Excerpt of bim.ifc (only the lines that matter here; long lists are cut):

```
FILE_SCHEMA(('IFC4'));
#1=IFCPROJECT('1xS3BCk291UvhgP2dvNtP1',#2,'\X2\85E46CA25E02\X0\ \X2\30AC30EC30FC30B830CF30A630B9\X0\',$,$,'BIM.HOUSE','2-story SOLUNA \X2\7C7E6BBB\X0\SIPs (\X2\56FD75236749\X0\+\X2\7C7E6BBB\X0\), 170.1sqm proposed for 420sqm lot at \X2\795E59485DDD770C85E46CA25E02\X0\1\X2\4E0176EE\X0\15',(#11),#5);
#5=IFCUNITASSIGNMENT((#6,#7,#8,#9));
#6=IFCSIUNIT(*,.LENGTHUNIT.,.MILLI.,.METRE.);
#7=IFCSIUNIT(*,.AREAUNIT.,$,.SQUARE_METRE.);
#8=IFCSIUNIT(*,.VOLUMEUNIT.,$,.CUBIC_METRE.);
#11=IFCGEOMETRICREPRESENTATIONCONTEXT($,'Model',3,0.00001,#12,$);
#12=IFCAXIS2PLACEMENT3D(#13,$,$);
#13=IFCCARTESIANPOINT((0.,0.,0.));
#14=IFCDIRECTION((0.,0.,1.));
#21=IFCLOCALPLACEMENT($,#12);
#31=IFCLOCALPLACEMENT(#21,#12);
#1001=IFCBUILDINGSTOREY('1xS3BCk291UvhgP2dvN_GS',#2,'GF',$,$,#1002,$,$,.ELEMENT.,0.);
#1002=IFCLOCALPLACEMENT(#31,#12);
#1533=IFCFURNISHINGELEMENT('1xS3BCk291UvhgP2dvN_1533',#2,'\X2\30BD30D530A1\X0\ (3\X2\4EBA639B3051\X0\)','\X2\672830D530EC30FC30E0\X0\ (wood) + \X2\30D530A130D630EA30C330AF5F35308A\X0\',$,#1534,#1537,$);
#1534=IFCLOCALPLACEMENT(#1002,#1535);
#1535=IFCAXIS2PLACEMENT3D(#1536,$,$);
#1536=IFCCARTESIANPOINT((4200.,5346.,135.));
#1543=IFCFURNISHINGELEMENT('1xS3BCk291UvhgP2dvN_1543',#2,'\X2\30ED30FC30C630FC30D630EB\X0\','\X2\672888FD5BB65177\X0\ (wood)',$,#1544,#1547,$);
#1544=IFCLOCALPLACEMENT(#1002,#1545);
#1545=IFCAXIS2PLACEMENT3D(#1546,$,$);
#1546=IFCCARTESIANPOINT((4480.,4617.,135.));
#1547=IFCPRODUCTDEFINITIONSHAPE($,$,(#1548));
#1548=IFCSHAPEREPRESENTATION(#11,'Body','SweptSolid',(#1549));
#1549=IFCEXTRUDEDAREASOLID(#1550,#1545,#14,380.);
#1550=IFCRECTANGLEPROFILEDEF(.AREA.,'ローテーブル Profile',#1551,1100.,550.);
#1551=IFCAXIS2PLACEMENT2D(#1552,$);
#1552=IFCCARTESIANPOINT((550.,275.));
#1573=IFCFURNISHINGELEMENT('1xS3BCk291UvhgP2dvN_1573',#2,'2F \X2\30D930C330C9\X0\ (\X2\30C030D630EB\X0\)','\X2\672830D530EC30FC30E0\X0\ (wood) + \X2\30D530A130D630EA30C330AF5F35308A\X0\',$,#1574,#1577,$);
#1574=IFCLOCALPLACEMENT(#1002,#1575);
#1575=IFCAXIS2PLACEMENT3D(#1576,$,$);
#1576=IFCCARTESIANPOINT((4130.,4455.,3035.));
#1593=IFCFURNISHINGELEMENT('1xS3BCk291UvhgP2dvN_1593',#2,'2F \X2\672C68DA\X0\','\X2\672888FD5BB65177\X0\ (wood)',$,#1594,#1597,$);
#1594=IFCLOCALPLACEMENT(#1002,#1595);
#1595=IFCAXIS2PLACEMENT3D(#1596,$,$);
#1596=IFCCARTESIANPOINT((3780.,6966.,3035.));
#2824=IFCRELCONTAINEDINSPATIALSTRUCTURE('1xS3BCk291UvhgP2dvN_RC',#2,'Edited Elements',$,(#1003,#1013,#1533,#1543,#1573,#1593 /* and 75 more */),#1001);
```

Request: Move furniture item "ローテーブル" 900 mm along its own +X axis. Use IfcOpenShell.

```python
import ifcopenshell
import ifcopenshell.api.geometry
import ifcopenshell.util.placement

model = ifcopenshell.open("bim.ifc")

item = model.by_guid("1xS3BCk291UvhgP2dvN_1543")
matrix = ifcopenshell.util.placement.get_local_placement(item.ObjectPlacement)
matrix[:3, 3] += matrix[:3, 0] * 900.0
ifcopenshell.api.geometry.edit_object_placement(model, product=item, matrix=matrix, is_si=False)

print(ifcopenshell.util.placement.get_local_placement(item.ObjectPlacement).round(3) + 0.0)

model.write("bim_updated.ifc")
```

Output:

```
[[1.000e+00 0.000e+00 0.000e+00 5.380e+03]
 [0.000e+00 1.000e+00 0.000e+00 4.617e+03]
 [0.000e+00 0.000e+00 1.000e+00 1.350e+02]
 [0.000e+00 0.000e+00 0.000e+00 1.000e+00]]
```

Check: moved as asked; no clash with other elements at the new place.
